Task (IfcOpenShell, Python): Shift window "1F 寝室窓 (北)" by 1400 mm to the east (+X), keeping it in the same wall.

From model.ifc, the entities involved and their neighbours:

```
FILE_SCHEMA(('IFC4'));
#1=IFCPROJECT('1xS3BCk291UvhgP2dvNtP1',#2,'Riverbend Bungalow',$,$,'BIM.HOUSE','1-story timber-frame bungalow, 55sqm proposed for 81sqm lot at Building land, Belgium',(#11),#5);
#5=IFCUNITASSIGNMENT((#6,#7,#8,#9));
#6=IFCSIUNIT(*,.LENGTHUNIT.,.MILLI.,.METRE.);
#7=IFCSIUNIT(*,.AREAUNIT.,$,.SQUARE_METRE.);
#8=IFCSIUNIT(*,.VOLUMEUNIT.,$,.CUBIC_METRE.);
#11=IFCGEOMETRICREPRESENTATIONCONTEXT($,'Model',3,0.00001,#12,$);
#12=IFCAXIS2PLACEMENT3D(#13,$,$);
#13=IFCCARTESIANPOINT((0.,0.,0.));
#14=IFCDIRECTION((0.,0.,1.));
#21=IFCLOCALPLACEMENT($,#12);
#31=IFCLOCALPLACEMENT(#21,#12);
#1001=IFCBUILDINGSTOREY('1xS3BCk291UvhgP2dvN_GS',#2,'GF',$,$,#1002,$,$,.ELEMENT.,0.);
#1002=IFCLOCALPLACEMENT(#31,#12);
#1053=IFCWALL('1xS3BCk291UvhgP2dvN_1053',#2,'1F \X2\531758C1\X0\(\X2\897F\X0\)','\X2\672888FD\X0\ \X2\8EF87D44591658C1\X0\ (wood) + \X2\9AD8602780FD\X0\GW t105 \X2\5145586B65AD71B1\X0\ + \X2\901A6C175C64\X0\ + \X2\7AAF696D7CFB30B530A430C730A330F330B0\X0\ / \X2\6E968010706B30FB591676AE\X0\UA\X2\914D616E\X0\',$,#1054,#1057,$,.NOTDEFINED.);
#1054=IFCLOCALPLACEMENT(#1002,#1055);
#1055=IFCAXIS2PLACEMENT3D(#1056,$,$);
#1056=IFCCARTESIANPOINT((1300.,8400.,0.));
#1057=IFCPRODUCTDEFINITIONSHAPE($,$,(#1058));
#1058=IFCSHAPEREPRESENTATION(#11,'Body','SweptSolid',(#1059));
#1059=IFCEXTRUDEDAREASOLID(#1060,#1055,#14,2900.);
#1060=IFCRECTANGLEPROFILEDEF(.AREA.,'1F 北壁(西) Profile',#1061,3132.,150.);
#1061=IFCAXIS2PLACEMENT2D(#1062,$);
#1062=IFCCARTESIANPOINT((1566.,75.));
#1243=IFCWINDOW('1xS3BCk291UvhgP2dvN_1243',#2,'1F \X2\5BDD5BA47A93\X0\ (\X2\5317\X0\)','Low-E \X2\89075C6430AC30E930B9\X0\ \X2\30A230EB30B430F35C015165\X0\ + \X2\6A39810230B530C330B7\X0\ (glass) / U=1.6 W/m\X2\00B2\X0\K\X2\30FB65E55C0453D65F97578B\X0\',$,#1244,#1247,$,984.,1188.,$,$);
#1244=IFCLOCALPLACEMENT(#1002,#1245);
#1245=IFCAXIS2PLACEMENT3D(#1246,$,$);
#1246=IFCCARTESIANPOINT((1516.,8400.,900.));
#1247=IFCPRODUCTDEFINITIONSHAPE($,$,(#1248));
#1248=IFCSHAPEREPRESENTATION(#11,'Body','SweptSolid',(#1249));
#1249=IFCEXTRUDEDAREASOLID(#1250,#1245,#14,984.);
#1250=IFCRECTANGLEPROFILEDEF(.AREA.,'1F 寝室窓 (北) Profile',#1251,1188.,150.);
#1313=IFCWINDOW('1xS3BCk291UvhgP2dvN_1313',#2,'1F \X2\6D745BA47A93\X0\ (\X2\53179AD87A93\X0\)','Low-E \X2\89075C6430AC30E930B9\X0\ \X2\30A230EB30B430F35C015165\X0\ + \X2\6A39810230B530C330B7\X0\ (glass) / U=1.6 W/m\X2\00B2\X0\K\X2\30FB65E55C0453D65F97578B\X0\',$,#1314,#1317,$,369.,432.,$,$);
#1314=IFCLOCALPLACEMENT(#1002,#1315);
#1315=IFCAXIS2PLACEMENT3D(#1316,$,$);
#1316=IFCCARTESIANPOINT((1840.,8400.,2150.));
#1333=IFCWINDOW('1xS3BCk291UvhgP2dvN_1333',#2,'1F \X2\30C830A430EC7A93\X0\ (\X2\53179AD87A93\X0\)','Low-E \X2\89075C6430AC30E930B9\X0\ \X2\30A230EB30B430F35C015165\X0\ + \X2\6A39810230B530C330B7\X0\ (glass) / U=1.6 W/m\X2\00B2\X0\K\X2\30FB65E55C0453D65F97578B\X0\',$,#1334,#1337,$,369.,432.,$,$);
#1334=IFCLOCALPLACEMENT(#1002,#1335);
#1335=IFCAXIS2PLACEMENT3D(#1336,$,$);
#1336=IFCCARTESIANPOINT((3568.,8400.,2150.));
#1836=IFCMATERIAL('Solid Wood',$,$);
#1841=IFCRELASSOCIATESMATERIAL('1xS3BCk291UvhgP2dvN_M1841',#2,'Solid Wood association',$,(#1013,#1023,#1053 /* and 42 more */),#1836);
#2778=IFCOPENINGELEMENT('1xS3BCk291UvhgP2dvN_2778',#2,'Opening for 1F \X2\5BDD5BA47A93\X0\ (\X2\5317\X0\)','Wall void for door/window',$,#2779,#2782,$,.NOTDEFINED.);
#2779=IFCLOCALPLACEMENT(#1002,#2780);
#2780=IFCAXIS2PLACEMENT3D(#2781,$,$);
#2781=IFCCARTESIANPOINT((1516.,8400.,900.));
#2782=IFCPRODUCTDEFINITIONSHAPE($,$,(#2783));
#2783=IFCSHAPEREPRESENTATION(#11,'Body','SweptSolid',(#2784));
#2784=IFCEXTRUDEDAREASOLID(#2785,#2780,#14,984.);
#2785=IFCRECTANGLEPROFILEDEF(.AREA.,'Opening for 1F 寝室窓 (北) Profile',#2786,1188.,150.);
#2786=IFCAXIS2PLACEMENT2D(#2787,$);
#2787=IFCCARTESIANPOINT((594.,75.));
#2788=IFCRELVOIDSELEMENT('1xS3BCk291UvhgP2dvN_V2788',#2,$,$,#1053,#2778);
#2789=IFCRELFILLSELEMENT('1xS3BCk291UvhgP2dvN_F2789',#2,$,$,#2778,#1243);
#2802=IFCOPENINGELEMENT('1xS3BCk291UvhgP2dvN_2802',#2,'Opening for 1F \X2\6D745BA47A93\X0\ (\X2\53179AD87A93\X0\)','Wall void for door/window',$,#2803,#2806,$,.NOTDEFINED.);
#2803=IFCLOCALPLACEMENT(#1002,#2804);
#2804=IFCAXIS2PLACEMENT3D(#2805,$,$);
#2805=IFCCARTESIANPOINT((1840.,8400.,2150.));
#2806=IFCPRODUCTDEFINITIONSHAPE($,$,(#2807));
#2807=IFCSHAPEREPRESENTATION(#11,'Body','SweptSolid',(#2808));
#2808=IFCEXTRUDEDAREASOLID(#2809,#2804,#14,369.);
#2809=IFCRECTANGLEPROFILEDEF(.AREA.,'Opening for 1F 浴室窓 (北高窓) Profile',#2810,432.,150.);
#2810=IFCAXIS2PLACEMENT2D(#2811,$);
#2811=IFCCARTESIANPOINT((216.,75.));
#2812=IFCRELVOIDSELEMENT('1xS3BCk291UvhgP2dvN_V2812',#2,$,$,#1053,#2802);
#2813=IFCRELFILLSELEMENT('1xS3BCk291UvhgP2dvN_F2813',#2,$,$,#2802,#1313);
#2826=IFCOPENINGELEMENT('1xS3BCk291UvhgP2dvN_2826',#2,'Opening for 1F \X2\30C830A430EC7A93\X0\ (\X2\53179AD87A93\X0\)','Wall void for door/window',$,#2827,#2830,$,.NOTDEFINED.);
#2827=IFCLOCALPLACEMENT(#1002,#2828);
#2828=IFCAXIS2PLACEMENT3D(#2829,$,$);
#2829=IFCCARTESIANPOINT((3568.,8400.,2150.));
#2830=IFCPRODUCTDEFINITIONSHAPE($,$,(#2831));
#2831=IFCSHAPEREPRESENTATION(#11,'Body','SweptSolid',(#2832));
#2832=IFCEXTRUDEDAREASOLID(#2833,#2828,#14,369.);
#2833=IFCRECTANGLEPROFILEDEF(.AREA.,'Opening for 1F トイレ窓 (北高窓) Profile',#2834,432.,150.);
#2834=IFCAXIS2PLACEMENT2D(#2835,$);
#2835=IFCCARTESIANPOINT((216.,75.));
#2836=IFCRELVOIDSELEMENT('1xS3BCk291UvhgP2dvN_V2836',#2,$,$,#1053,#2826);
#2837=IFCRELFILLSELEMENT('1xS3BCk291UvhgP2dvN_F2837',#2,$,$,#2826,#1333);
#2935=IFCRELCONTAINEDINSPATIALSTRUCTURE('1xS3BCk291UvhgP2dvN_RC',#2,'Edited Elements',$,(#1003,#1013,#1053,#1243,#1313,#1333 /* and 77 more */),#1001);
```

```python
import ifcopenshell
import ifcopenshell.api.geometry
import ifcopenshell.util.placement
import ifcopenshell.util.unit

model = ifcopenshell.open("model.ifc")
unit_scale = ifcopenshell.util.unit.calculate_unit_scale(model)

window = model.by_guid("1xS3BCk291UvhgP2dvN_1243")
opening = window.FillsVoids[0].RelatingOpeningElement
wall = opening.VoidsElements[0].RelatingBuildingElement

wall_matrix = ifcopenshell.util.placement.get_local_placement(wall.ObjectPlacement)
shift = wall_matrix[:3, 0] * 1.4 / unit_scale
before = ifcopenshell.util.placement.get_local_placement(window.ObjectPlacement)[:3, 3].copy()

# The window is not placed relative to its opening, so move both.
for product in (opening, window):
    matrix = ifcopenshell.util.placement.get_local_placement(product.ObjectPlacement)
    matrix[:3, 3] += shift
    ifcopenshell.api.geometry.edit_object_placement(model, product=product, matrix=matrix, is_si=False)

after = ifcopenshell.util.placement.get_local_placement(window.ObjectPlacement)[:3, 3]
print("window moved by", (after - before).round(3) + 0.0)

model.write("model-out.ifc")
```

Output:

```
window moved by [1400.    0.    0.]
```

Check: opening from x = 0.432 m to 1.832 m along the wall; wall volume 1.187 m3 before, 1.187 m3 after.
